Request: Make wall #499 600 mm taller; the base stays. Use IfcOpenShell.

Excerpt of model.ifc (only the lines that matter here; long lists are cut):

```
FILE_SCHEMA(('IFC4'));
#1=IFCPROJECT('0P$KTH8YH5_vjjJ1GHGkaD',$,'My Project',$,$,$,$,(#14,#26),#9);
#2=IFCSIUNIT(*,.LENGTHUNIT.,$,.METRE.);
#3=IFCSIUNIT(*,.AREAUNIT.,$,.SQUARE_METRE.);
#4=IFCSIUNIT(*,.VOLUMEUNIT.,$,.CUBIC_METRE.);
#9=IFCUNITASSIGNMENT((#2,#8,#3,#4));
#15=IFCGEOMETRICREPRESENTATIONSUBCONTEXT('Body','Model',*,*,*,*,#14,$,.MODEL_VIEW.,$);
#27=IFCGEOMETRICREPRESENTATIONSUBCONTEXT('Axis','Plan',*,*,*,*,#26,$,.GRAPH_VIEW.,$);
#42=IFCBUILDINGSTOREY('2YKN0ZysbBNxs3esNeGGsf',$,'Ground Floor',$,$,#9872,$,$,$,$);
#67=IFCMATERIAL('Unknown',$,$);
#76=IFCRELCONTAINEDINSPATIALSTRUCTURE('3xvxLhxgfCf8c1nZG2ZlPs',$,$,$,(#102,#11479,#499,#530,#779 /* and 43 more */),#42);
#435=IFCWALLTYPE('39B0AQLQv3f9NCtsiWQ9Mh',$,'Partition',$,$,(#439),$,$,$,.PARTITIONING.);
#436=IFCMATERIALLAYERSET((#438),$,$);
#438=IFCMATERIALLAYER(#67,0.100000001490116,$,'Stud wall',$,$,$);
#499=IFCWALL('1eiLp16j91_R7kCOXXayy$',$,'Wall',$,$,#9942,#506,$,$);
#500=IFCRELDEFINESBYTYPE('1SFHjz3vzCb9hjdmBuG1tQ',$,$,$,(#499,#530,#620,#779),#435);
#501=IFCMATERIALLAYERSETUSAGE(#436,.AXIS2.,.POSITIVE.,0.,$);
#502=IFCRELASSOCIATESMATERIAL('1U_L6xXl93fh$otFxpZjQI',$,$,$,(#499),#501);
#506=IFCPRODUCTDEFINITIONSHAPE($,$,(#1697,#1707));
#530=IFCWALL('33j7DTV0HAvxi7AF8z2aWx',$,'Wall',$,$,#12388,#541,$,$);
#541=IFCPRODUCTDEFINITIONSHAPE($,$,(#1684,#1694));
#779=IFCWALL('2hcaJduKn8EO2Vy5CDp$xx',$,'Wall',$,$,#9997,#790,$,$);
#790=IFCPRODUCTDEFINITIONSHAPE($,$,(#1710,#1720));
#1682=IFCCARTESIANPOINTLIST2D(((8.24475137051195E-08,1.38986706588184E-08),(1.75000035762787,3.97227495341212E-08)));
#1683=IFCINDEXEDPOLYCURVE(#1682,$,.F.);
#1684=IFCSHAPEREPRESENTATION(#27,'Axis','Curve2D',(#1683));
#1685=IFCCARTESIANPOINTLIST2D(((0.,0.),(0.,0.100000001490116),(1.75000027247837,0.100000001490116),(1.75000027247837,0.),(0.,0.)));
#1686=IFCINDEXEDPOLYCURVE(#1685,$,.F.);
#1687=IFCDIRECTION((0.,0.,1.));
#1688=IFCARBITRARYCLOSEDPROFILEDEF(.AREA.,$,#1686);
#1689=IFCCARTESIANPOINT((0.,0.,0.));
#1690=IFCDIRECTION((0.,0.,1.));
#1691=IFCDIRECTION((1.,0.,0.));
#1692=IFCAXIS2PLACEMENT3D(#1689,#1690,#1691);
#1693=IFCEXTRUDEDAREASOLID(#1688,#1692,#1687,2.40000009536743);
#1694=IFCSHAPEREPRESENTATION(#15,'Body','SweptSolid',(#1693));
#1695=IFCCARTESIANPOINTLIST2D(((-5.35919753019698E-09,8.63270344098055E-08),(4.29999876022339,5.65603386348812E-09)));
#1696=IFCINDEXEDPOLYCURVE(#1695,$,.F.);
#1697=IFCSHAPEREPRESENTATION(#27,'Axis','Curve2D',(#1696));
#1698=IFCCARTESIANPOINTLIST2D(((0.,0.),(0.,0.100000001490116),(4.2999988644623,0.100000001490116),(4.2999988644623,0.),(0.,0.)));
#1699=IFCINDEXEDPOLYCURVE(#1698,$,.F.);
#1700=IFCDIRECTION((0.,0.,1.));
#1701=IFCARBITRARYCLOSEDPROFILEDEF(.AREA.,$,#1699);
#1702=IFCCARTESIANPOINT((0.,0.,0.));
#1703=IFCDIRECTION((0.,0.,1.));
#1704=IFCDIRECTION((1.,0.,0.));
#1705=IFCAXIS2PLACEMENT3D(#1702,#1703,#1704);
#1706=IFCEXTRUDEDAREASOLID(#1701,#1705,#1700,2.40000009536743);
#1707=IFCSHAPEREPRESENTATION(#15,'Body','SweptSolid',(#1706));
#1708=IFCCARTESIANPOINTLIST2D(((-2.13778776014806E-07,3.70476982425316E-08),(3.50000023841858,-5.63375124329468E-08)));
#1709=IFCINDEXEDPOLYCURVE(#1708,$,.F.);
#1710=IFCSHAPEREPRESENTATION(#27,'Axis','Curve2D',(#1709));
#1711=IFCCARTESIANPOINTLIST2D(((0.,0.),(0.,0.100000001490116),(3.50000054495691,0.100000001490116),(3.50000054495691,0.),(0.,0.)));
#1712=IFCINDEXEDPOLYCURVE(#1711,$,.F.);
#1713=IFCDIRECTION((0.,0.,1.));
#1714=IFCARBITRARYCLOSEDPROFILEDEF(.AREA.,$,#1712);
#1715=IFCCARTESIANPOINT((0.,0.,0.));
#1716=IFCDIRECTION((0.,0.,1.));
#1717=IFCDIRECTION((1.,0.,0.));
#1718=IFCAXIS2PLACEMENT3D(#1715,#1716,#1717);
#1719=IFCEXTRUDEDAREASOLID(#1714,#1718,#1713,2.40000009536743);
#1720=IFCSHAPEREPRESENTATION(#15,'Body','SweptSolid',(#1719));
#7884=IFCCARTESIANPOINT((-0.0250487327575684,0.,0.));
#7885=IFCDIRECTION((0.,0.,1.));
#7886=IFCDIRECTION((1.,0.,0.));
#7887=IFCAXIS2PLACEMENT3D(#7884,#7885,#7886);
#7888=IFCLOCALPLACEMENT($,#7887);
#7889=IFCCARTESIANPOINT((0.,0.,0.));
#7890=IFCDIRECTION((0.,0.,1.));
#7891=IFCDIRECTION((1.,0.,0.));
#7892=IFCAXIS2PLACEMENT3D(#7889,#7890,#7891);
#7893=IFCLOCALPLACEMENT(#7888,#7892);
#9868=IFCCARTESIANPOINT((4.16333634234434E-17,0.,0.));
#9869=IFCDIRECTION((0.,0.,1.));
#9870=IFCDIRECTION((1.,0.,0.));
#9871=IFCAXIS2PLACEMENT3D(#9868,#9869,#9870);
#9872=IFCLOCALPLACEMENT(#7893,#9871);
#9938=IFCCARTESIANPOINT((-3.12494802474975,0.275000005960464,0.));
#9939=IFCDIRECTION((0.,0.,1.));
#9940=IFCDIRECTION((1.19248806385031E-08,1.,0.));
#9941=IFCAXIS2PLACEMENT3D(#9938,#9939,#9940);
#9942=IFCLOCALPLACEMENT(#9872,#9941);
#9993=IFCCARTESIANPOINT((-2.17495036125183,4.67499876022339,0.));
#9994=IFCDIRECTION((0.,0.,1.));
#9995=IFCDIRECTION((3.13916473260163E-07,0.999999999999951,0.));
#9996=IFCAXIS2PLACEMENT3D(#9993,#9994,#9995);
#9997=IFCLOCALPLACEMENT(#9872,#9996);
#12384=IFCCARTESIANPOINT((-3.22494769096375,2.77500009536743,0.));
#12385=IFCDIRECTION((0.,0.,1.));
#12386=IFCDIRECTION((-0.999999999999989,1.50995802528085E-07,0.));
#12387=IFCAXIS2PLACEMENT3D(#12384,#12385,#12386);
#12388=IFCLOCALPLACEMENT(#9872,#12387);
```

```python
import ifcopenshell
import ifcopenshell.geom
import ifcopenshell.util.representation
import ifcopenshell.util.shape
import ifcopenshell.util.unit

model = ifcopenshell.open("model.ifc")
unit_scale = ifcopenshell.util.unit.calculate_unit_scale(model)
settings = ifcopenshell.geom.settings()


def volume(element):
    """Net volume in cubic metres, openings subtracted."""
    shape = ifcopenshell.geom.create_shape(settings, element)
    return ifcopenshell.util.shape.get_volume(shape.geometry)


wall = model.by_id(499)
before = volume(wall)

body = ifcopenshell.util.representation.get_representation(wall, "Model", "Body")
solid = body.Items[0]
old_height = solid.Depth
solid.Depth += 0.6 / unit_scale
after = volume(wall)

print(f"height {old_height:g} -> {solid.Depth:g}, volume {before:.3f} -> {after:.3f} m3")

model.write("model-out.ifc")
```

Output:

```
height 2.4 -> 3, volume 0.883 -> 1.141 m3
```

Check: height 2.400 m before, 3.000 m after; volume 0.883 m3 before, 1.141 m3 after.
